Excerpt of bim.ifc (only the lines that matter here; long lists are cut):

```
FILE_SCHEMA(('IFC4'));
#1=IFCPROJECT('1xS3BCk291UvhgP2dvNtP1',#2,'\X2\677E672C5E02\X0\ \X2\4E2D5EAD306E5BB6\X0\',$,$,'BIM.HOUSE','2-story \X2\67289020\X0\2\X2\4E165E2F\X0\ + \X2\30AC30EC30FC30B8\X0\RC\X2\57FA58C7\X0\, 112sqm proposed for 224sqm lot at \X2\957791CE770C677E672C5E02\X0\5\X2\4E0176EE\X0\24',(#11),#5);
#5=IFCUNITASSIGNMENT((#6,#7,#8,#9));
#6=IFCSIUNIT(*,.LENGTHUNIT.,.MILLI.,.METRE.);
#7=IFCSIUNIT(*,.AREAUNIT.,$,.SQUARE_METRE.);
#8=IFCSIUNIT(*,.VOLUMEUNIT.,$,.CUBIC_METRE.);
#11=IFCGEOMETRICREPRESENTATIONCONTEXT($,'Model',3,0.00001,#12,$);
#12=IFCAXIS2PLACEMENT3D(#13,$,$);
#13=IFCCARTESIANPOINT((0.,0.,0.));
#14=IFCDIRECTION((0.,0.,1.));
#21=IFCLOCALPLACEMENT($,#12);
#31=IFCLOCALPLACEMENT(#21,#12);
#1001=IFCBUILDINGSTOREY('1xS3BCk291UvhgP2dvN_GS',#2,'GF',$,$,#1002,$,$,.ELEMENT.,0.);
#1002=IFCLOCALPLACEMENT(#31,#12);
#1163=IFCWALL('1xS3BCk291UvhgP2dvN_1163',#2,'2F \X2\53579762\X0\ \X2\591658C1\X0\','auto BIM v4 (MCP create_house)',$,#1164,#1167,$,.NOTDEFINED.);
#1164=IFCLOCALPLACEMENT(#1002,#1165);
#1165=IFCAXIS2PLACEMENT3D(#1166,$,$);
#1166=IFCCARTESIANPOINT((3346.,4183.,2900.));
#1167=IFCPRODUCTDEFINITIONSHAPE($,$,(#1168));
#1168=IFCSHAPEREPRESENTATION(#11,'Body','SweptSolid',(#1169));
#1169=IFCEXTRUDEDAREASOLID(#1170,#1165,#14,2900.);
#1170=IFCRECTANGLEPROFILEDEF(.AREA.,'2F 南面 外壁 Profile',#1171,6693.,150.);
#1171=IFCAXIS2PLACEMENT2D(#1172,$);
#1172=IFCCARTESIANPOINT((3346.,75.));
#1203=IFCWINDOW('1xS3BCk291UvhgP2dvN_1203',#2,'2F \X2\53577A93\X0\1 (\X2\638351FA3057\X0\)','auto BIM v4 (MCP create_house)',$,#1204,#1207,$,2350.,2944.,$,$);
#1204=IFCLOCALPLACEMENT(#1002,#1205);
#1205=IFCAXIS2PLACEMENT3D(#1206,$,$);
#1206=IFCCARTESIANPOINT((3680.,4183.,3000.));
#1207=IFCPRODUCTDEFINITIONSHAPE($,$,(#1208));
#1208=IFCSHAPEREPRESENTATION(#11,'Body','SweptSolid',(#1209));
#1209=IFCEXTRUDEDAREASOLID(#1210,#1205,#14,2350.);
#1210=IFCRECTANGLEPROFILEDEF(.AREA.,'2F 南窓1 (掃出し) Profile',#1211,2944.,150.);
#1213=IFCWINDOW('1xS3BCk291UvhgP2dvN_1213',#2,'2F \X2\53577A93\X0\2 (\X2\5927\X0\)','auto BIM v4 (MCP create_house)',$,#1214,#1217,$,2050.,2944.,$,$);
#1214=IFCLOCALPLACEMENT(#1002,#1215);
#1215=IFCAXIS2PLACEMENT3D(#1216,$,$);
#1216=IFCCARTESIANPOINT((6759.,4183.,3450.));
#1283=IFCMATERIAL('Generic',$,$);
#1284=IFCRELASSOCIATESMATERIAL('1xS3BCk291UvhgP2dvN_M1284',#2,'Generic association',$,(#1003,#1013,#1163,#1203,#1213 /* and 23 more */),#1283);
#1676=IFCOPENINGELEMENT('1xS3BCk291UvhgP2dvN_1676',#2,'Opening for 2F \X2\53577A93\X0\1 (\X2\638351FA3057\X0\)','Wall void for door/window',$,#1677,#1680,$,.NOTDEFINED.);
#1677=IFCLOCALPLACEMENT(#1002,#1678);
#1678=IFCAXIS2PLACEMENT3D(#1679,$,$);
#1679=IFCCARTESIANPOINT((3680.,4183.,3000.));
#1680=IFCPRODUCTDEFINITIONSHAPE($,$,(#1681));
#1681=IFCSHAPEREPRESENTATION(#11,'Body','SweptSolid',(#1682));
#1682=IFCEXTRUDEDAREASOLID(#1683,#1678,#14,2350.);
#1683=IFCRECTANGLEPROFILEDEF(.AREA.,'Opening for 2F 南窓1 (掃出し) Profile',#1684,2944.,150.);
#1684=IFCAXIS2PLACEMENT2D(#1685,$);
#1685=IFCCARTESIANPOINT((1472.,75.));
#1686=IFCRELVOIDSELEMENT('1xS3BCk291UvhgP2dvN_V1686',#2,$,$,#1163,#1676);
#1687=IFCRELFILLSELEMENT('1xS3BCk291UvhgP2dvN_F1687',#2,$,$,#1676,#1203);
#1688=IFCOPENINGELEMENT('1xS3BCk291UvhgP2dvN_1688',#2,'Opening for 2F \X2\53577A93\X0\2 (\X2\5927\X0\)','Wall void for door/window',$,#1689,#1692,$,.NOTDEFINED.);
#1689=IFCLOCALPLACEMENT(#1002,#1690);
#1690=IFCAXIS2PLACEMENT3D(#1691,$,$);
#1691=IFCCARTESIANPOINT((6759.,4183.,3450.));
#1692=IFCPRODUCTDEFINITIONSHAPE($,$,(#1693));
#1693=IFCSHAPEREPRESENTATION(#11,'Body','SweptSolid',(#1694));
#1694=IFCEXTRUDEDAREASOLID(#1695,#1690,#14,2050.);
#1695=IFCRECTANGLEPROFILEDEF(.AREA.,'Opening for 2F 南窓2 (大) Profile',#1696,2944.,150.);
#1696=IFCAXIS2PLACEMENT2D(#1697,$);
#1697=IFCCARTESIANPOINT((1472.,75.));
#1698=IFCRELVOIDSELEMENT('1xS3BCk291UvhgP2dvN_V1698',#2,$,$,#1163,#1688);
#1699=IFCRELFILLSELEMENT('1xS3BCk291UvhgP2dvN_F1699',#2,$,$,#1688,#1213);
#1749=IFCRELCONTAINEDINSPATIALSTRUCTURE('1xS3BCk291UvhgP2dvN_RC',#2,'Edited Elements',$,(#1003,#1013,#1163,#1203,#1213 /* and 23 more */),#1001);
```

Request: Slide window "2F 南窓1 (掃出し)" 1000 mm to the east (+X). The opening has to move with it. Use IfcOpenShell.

```python
import ifcopenshell
import ifcopenshell.api.geometry
import ifcopenshell.util.placement

model = ifcopenshell.open("bim.ifc")

window = model.by_guid("1xS3BCk291UvhgP2dvN_1203")
opening = window.FillsVoids[0].RelatingOpeningElement
wall = opening.VoidsElements[0].RelatingBuildingElement

wall_matrix = ifcopenshell.util.placement.get_local_placement(wall.ObjectPlacement)
shift = wall_matrix[:3, 0] * 1000.0
before = ifcopenshell.util.placement.get_local_placement(window.ObjectPlacement)[:3, 3].copy()

# The window is not placed relative to its opening, so move both.
for product in (opening, window):
    matrix = ifcopenshell.util.placement.get_local_placement(product.ObjectPlacement)
    matrix[:3, 3] += shift
    ifcopenshell.api.geometry.edit_object_placement(model, product=product, matrix=matrix, is_si=False)

after = ifcopenshell.util.placement.get_local_placement(window.ObjectPlacement)[:3, 3]
print("window moved by", (after - before).round(3) + 0.0)

model.write("bim_edited.ifc")
```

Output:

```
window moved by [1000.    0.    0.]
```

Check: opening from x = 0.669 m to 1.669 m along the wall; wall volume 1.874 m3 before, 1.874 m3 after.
